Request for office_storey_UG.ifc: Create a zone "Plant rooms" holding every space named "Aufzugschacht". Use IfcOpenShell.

First a look at what the model holds.

```python
import ifcopenshell

model = ifcopenshell.open("office_storey_UG.ifc")
print(model.schema)
seen = {}
for space in model.by_type("IfcSpace"):
    seen[space.LongName] = seen.get(space.LongName, 0) + 1
for name, count in sorted(seen.items(), key=str):
    print(count, "x", name)
print("zones:", [z.Name for z in model.by_type("IfcZone")][:20])
```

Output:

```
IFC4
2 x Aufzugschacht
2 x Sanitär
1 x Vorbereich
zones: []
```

```python
import ifcopenshell
import ifcopenshell.api.group
import ifcopenshell.api.root

model = ifcopenshell.open("office_storey_UG.ifc")

names = {"Aufzugschacht"}
spaces = [s for s in model.by_type("IfcSpace") if s.LongName in names]

zone = ifcopenshell.api.root.create_entity(model, ifc_class="IfcZone", name="Plant rooms")
ifcopenshell.api.group.assign_group(model, products=spaces, group=zone)
print(len(spaces), "spaces in", zone.Name)

model.write("office_storey_UG_rev.ifc")
```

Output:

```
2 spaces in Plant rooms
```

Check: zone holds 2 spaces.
